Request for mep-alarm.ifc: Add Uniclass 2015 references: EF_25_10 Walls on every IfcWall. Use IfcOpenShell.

First a look at what the model holds.

```python
import ifcopenshell

model = ifcopenshell.open("mep-alarm.ifc")
print(model.schema)
print("classifications:", [c.Name for c in model.by_type("IfcClassification")])
for ifc_class in ("IfcDoor", "IfcRoof", "IfcStair", "IfcWall", "IfcWindow"):
    print(ifc_class, len(model.by_type(ifc_class)))
```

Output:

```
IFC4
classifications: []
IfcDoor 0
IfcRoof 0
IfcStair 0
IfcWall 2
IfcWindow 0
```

```python
import ifcopenshell
import ifcopenshell.api.classification

model = ifcopenshell.open("mep-alarm.ifc")

system = ifcopenshell.api.classification.add_classification(model, classification="Uniclass 2015")

codes = {
    "IfcWall": ("EF_25_10", "Walls"),
}
for ifc_class, (code, name) in codes.items():
    products = model.by_type(ifc_class)
    ifcopenshell.api.classification.add_reference(
        model, products=products, classification=system, identification=code, name=name
    )
    print(code, len(products))

model.write("mep-alarm_updated.ifc")
```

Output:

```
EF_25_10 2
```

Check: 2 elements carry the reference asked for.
